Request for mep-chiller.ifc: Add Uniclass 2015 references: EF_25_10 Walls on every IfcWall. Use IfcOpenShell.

First a look at what the model holds.

```python
import ifcopenshell

model = ifcopenshell.open("mep-chiller.ifc")
print(model.schema)
print("classifications:", [c.Name for c in model.by_type("IfcClassification")])
for ifc_class in ("IfcDoor", "IfcRoof", "IfcStair", "IfcWall", "IfcWindow"):
    print(ifc_class, len(model.by_type(ifc_class)))
```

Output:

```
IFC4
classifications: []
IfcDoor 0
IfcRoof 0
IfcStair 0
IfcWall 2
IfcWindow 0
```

```python
import ifcopenshell
import ifcopenshell.api.classification

model = ifcopenshell.open("mep-chiller.ifc")

system = ifcopenshell.api.classification.add_classification(model, classification="Uniclass 2015")

codes = {
    "IfcWall": ("EF_25_10", "Walls"),
}
for ifc_class, (code, name) in codes.items():
    products = model.by_type(ifc_class)
    ifcopenshell.api.classification.add_reference(
        model, products=products, classification=system, identification=code, name=name
    )
    print(code, len(products))

model.write("mep-chiller_rev.ifc")
```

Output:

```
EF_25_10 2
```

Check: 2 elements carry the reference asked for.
